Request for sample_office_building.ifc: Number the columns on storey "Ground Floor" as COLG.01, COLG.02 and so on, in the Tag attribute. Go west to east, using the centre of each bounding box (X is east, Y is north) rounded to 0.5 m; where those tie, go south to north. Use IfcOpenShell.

First a look at what the model holds.

```python
import ifcopenshell
import ifcopenshell.util.element
import ifcopenshell.util.placement

model = ifcopenshell.open("sample_office_building.ifc")
print(model.schema)
storey = next(s for s in model.by_type("IfcBuildingStorey") if s.Name == "Ground Floor")
columns = [e for e in ifcopenshell.util.element.get_decomposition(storey) if e.is_a("IfcColumn")]
for e in sorted(columns, key=lambda e: e.id()):
    origin = ifcopenshell.util.placement.get_local_placement(e.ObjectPlacement)[:3, 3]
    print(e.id(), e.Tag, e.Name, origin.round(2) + 0.0, sep=" | ")
```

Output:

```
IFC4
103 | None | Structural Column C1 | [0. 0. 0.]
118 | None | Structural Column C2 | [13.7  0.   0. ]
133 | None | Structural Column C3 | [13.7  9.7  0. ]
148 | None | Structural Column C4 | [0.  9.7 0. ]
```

```python
import ifcopenshell
import ifcopenshell.geom
import ifcopenshell.util.element
import ifcopenshell.util.shape

model = ifcopenshell.open("sample_office_building.ifc")
settings = ifcopenshell.geom.settings()
settings.set("use-world-coords", True)


def centre(element):
    shape = ifcopenshell.geom.create_shape(settings, element)
    return ifcopenshell.util.shape.get_bbox_centroid(shape.geometry)


storey = next(s for s in model.by_type("IfcBuildingStorey") if s.Name == "Ground Floor")
columns = [e for e in ifcopenshell.util.element.get_decomposition(storey) if e.is_a("IfcColumn")]

# Insertion points can sit at a corner or the storey origin, so sort by the geometry (in metres).
centres = {e: centre(e) for e in columns}
columns.sort(key=lambda e: (round(centres[e][0] / 0.5), centres[e][1]))

for i, e in enumerate(columns, start=1):
    number = f"COLG.{i:02d}"
    e.Tag = number
    print(e.id(), number)

model.write("sample_office_building_rev.ifc")
```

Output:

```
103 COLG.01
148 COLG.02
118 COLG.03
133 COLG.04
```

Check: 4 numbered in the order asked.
